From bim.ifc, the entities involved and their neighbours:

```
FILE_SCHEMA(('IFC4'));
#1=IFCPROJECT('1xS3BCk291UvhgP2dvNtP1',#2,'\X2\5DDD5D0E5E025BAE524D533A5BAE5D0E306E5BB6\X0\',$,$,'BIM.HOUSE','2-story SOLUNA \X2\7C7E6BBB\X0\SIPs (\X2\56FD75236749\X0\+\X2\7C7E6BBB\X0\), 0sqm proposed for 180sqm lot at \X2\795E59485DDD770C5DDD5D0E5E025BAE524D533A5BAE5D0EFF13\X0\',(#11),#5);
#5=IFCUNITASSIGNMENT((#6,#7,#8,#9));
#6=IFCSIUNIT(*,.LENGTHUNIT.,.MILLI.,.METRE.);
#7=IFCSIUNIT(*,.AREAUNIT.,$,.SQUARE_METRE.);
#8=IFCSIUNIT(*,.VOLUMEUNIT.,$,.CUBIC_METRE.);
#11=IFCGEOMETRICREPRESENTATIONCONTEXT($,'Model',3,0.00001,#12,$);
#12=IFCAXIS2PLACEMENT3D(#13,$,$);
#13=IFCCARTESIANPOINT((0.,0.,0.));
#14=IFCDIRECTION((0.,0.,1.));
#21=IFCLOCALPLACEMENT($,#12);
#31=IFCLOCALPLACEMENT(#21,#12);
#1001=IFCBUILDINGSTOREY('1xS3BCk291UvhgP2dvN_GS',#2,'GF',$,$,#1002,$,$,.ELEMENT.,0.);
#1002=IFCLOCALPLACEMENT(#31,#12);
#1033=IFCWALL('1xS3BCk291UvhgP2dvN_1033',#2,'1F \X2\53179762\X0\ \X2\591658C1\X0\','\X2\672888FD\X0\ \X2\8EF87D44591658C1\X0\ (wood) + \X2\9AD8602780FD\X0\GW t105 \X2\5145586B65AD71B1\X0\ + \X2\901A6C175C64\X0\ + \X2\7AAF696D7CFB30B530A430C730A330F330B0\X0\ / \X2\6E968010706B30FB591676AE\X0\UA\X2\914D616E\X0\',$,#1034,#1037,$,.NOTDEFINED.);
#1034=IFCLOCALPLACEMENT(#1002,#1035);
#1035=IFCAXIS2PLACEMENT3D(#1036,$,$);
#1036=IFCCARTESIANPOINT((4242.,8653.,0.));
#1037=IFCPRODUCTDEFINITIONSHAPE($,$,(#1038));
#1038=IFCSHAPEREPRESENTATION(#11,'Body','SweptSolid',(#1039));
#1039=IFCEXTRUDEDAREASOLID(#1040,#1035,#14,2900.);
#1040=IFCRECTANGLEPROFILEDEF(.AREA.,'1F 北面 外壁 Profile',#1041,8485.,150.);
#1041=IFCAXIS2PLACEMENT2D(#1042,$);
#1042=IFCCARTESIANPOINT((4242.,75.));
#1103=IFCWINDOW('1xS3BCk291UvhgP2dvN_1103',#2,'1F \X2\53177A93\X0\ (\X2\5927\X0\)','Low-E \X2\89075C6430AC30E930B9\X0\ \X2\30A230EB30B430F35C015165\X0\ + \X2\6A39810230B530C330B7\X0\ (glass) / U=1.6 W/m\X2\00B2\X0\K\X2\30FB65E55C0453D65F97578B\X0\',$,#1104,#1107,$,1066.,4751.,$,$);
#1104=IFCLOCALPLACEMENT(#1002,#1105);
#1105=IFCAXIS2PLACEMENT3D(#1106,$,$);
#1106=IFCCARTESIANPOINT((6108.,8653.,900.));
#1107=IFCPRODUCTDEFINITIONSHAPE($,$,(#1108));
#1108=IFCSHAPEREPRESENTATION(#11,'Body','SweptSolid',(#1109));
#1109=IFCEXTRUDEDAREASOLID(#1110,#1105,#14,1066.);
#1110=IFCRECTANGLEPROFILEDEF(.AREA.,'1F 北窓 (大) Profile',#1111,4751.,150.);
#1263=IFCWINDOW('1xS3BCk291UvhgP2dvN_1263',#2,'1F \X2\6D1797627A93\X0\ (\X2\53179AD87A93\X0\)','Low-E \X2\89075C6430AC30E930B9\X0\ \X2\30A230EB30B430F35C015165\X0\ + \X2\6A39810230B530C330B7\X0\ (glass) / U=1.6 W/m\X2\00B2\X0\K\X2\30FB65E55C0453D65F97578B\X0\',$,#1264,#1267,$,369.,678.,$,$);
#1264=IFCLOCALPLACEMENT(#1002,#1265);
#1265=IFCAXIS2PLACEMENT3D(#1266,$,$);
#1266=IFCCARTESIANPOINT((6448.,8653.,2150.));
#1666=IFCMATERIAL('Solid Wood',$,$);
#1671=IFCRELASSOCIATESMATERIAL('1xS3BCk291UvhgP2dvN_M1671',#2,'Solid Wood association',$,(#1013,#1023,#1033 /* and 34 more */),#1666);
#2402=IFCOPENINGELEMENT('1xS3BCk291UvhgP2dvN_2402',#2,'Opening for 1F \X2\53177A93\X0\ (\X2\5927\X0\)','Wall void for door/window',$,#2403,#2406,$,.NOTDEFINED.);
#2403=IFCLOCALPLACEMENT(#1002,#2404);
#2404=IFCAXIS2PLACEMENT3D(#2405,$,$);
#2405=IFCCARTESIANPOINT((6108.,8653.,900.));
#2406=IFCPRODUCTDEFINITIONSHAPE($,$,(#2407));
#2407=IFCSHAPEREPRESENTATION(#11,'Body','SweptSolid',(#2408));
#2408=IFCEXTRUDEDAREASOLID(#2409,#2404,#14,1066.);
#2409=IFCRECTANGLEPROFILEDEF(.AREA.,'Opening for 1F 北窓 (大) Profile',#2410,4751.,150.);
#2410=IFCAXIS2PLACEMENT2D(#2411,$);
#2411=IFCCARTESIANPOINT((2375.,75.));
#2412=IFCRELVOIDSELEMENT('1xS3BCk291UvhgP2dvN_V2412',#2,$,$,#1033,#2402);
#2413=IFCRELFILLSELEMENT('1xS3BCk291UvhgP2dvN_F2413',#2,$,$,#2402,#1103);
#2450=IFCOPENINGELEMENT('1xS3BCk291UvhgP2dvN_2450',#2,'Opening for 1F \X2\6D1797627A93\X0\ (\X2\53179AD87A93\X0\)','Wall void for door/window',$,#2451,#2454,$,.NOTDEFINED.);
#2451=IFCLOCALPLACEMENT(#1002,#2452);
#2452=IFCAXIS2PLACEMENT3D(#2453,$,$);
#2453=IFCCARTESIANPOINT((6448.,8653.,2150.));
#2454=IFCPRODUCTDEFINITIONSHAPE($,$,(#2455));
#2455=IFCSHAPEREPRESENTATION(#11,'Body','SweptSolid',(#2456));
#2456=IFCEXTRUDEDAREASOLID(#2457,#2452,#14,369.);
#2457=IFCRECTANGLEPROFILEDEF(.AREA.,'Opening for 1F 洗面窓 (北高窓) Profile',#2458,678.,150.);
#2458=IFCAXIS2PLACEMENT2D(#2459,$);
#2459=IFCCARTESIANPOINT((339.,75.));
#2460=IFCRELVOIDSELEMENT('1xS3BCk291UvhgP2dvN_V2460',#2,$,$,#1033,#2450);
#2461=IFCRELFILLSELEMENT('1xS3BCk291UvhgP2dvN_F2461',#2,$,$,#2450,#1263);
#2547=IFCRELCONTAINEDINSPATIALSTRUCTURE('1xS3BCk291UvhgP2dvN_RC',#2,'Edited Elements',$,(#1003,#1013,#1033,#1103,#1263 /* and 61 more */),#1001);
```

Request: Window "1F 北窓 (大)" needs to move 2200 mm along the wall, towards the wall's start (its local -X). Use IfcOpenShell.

```python
import ifcopenshell
import ifcopenshell.api.geometry
import ifcopenshell.util.placement
import ifcopenshell.util.unit

model = ifcopenshell.open("bim.ifc")
unit_scale = ifcopenshell.util.unit.calculate_unit_scale(model)

window = model.by_guid("1xS3BCk291UvhgP2dvN_1103")
opening = window.FillsVoids[0].RelatingOpeningElement
wall = opening.VoidsElements[0].RelatingBuildingElement

wall_matrix = ifcopenshell.util.placement.get_local_placement(wall.ObjectPlacement)
shift = wall_matrix[:3, 0] * -2.2 / unit_scale
before = ifcopenshell.util.placement.get_local_placement(window.ObjectPlacement)[:3, 3].copy()

# The window is not placed relative to its opening, so move both.
for product in (opening, window):
    matrix = ifcopenshell.util.placement.get_local_placement(product.ObjectPlacement)
    matrix[:3, 3] += shift
    ifcopenshell.api.geometry.edit_object_placement(model, product=product, matrix=matrix, is_si=False)

after = ifcopenshell.util.placement.get_local_placement(window.ObjectPlacement)[:3, 3]
print("window moved by", (after - before).round(3) + 0.0)

model.write("bim_edited.ifc")
```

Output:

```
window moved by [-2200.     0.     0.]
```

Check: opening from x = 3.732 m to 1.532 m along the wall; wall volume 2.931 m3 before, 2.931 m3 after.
